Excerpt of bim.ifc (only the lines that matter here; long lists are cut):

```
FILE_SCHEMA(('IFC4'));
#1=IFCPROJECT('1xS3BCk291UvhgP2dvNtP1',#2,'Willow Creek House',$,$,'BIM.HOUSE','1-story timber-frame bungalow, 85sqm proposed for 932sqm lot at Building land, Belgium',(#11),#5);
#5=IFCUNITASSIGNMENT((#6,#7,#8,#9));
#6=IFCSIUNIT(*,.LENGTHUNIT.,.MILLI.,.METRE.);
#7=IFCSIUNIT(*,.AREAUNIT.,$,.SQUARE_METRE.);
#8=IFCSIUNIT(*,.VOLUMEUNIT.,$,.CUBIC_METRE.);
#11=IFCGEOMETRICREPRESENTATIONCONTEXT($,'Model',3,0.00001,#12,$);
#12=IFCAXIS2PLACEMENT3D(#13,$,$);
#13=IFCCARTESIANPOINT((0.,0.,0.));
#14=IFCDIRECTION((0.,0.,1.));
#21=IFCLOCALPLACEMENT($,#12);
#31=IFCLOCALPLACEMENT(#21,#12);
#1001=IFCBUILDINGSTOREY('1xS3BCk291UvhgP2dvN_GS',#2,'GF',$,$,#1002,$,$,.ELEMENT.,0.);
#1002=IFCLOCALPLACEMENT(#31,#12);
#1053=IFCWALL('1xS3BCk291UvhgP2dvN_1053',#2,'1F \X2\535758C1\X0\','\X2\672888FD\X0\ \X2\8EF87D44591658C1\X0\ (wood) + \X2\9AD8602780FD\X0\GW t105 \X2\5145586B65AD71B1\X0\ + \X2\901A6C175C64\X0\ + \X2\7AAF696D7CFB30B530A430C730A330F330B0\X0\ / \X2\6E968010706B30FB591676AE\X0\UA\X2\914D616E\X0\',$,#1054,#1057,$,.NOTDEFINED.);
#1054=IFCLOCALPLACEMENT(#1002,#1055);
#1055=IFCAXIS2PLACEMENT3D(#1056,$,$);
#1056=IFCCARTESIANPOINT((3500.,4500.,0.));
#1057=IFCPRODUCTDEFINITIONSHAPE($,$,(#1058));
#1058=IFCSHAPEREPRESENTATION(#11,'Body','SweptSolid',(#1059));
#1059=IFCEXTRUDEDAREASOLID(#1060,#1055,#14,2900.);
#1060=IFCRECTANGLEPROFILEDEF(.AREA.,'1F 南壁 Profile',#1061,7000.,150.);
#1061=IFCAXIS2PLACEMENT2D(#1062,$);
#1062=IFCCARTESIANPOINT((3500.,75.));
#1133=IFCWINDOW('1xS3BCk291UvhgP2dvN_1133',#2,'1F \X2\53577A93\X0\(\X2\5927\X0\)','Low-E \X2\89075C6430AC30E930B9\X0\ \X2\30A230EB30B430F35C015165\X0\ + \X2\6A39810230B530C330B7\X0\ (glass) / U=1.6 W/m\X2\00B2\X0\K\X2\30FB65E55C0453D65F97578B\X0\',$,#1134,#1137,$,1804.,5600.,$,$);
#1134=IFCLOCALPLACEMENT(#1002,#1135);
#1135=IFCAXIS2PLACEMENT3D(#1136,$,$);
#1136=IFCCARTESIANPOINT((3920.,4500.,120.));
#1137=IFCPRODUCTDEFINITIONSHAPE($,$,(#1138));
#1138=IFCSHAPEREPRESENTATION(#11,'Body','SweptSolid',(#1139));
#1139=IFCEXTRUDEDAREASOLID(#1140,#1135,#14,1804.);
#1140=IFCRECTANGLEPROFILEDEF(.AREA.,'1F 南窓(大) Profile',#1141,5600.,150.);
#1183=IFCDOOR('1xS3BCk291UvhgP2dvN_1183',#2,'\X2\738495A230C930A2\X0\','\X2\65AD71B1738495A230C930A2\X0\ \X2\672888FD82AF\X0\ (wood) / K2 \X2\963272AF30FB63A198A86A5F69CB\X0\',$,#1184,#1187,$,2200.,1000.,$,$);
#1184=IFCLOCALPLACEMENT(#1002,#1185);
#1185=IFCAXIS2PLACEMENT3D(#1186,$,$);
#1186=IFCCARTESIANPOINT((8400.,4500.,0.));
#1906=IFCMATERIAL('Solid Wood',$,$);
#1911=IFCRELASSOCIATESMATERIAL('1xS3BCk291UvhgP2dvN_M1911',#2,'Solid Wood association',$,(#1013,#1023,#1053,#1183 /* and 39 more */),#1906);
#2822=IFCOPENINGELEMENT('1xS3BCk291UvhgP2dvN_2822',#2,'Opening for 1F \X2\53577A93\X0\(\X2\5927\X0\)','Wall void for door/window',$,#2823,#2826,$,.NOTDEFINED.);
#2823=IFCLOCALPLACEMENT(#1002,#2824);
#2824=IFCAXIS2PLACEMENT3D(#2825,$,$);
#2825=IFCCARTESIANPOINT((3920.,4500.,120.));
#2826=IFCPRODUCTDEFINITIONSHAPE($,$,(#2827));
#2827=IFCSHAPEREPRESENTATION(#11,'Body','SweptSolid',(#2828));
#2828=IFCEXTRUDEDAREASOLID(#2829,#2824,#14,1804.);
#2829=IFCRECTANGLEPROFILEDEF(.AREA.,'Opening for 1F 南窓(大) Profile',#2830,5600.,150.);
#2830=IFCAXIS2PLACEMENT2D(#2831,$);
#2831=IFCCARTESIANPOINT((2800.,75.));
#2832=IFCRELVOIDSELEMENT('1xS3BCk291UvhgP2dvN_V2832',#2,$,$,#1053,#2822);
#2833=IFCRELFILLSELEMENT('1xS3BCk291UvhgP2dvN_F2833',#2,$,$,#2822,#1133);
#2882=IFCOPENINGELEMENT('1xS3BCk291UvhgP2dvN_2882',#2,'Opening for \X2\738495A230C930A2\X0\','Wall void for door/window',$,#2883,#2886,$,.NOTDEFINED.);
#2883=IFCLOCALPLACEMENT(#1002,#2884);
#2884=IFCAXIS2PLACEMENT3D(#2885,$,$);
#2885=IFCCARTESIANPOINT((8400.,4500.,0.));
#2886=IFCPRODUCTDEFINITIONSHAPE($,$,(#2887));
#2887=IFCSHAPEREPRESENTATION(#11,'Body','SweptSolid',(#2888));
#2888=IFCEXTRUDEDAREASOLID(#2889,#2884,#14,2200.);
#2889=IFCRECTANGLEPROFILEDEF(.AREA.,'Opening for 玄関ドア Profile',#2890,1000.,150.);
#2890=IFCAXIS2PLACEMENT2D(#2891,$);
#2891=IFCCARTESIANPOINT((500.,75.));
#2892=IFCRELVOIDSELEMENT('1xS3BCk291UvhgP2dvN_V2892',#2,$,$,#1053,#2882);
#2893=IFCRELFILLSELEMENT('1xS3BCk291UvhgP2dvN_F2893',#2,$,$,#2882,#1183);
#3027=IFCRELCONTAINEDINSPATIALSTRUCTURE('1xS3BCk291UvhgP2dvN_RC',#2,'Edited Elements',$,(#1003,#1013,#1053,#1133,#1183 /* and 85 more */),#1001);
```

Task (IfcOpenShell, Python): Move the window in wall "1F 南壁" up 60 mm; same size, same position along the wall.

```python
import numpy as np
import ifcopenshell
import ifcopenshell.api.geometry
import ifcopenshell.util.placement
import ifcopenshell.util.unit

model = ifcopenshell.open("bim.ifc")
unit_scale = ifcopenshell.util.unit.calculate_unit_scale(model)

window = model.by_id(1133)
opening = window.FillsVoids[0].RelatingOpeningElement
dz = 0.06 / unit_scale

shift = np.array([0.0, 0.0, dz])
# The window is not placed relative to its opening, so move both.
for product in (opening, window):
    matrix = ifcopenshell.util.placement.get_local_placement(product.ObjectPlacement)
    matrix[:3, 3] += shift
    ifcopenshell.api.geometry.edit_object_placement(model, product=product, matrix=matrix, is_si=False)

print(f"moved by {dz * unit_scale:+.3f} m")

model.write("bim_v2.ifc")
```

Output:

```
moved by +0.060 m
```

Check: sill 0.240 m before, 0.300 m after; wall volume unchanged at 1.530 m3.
